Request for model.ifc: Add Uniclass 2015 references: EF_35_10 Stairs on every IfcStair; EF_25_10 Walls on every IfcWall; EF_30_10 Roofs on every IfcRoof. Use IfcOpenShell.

First a look at what the model holds.

```python
import ifcopenshell

model = ifcopenshell.open("model.ifc")
print(model.schema)
print("classifications:", [c.Name for c in model.by_type("IfcClassification")])
for ifc_class in ("IfcDoor", "IfcRoof", "IfcStair", "IfcWall", "IfcWindow"):
    print(ifc_class, len(model.by_type(ifc_class)))
```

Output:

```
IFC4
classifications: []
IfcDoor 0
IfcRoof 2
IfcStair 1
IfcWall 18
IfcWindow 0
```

```python
import ifcopenshell
import ifcopenshell.api.classification

model = ifcopenshell.open("model.ifc")

system = ifcopenshell.api.classification.add_classification(model, classification="Uniclass 2015")

codes = {
    "IfcStair": ("EF_35_10", "Stairs"),
    "IfcWall": ("EF_25_10", "Walls"),
    "IfcRoof": ("EF_30_10", "Roofs"),
}
for ifc_class, (code, name) in codes.items():
    products = model.by_type(ifc_class)
    ifcopenshell.api.classification.add_reference(
        model, products=products, classification=system, identification=code, name=name
    )
    print(code, len(products))

model.write("model_v2.ifc")
```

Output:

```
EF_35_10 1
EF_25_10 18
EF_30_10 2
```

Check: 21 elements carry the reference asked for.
